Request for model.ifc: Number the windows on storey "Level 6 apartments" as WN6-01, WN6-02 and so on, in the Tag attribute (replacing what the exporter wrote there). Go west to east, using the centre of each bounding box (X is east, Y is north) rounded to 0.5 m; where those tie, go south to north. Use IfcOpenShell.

First a look at what the model holds.

```python
import ifcopenshell
import ifcopenshell.util.element
import ifcopenshell.util.placement

model = ifcopenshell.open("model.ifc")
print(model.schema)
storey = next(s for s in model.by_type("IfcBuildingStorey") if s.Name == "Level 6 apartments")
windows = [e for e in ifcopenshell.util.element.get_decomposition(storey) if e.is_a("IfcWindow")]
for e in sorted(windows, key=lambda e: e.id()):
    origin = ifcopenshell.util.placement.get_local_placement(e.ObjectPlacement)[:3, 3]
    print(e.id(), e.Tag, e.Name, origin.round(2) + 0.0, sep=" | ")
```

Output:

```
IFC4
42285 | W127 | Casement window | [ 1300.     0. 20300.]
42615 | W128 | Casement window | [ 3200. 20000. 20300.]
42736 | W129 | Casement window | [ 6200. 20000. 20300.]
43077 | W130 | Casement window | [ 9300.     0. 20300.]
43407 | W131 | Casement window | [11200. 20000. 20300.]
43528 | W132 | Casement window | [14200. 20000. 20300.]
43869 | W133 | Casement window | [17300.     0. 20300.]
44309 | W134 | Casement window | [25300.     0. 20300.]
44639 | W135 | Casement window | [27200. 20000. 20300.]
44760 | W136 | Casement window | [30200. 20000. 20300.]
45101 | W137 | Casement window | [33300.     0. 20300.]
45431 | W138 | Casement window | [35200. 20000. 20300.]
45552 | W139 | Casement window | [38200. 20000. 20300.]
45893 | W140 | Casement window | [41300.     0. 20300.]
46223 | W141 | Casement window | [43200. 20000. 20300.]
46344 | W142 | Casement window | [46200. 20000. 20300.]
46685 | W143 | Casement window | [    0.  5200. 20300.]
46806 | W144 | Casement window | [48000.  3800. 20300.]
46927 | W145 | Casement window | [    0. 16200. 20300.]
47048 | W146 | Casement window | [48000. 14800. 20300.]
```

```python
import ifcopenshell
import ifcopenshell.geom
import ifcopenshell.util.element
import ifcopenshell.util.shape

model = ifcopenshell.open("model.ifc")
settings = ifcopenshell.geom.settings()
settings.set("use-world-coords", True)


def centre(element):
    shape = ifcopenshell.geom.create_shape(settings, element)
    return ifcopenshell.util.shape.get_bbox_centroid(shape.geometry)


storey = next(s for s in model.by_type("IfcBuildingStorey") if s.Name == "Level 6 apartments")
windows = [e for e in ifcopenshell.util.element.get_decomposition(storey) if e.is_a("IfcWindow")]

# Insertion points can sit at a corner or the storey origin, so sort by the geometry (in metres).
centres = {e: centre(e) for e in windows}
windows.sort(key=lambda e: (round(centres[e][0] / 0.5), centres[e][1]))

for i, e in enumerate(windows, start=1):
    number = f"WN6-{i:02d}"
    e.Tag = number
    print(e.id(), number)

model.write("model-out.ifc")
```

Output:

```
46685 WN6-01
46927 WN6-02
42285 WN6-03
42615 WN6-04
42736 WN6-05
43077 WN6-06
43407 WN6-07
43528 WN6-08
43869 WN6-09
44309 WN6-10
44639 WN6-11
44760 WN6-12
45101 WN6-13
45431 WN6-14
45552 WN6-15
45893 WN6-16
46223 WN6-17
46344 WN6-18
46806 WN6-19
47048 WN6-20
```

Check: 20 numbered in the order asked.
